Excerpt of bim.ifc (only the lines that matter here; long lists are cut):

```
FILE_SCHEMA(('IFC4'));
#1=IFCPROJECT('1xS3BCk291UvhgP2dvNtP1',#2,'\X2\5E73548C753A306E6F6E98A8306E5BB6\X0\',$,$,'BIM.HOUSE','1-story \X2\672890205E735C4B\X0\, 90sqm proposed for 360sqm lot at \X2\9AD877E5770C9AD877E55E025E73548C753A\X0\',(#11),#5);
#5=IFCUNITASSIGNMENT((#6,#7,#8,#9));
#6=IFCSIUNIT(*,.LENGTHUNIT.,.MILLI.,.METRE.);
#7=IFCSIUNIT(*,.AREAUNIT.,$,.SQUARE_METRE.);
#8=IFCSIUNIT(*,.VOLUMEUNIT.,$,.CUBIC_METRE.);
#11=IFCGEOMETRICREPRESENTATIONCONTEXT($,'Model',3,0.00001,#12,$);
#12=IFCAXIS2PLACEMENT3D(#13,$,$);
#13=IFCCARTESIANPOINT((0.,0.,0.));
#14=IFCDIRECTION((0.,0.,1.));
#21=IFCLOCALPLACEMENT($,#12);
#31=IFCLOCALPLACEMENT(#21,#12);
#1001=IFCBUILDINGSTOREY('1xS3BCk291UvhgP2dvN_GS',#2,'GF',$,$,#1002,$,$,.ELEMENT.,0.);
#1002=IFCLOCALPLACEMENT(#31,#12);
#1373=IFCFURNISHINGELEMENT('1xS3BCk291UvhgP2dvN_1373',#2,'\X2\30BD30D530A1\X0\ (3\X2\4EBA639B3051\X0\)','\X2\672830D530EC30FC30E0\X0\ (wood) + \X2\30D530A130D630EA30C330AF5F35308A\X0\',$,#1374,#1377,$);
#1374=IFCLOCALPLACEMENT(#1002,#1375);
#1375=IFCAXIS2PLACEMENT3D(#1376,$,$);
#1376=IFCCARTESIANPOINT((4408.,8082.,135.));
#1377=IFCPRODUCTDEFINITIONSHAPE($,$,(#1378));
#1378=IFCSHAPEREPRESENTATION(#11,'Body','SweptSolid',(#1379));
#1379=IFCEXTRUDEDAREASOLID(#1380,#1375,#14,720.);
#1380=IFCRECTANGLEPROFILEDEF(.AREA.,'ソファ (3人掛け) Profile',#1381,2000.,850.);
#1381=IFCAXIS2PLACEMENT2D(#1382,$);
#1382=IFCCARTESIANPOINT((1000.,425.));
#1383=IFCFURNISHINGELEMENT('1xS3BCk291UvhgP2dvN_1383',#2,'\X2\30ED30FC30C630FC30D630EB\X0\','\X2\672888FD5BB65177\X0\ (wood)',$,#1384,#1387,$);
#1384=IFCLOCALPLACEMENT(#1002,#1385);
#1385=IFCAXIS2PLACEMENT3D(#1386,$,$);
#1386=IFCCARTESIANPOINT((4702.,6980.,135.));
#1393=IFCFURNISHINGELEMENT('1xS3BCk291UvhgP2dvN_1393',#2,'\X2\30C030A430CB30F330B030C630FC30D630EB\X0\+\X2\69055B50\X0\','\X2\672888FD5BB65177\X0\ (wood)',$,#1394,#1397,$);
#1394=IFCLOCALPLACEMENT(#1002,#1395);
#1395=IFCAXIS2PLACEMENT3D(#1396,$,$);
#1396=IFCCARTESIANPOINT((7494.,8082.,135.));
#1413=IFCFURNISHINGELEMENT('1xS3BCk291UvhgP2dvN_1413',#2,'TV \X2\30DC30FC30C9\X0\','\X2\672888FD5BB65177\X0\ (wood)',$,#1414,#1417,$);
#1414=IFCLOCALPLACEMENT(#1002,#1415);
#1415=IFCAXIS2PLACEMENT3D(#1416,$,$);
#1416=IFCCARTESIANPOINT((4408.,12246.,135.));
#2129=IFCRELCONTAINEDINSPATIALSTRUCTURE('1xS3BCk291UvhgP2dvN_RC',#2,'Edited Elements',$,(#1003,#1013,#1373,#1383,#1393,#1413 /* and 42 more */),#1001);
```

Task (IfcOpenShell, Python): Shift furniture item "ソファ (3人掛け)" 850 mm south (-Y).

```python
import ifcopenshell
import ifcopenshell.api.geometry
import ifcopenshell.util.placement
import ifcopenshell.util.unit

model = ifcopenshell.open("bim.ifc")
unit_scale = ifcopenshell.util.unit.calculate_unit_scale(model)

item = model.by_id(1373)
matrix = ifcopenshell.util.placement.get_local_placement(item.ObjectPlacement)
matrix[1, 3] -= 0.85 / unit_scale
ifcopenshell.api.geometry.edit_object_placement(model, product=item, matrix=matrix, is_si=False)

print(ifcopenshell.util.placement.get_local_placement(item.ObjectPlacement).round(3) + 0.0)

model.write("bim_v2.ifc")
```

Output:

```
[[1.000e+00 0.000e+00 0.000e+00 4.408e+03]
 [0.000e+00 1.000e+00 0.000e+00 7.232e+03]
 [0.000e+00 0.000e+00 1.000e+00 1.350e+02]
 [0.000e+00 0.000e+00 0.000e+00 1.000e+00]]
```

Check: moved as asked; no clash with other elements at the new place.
